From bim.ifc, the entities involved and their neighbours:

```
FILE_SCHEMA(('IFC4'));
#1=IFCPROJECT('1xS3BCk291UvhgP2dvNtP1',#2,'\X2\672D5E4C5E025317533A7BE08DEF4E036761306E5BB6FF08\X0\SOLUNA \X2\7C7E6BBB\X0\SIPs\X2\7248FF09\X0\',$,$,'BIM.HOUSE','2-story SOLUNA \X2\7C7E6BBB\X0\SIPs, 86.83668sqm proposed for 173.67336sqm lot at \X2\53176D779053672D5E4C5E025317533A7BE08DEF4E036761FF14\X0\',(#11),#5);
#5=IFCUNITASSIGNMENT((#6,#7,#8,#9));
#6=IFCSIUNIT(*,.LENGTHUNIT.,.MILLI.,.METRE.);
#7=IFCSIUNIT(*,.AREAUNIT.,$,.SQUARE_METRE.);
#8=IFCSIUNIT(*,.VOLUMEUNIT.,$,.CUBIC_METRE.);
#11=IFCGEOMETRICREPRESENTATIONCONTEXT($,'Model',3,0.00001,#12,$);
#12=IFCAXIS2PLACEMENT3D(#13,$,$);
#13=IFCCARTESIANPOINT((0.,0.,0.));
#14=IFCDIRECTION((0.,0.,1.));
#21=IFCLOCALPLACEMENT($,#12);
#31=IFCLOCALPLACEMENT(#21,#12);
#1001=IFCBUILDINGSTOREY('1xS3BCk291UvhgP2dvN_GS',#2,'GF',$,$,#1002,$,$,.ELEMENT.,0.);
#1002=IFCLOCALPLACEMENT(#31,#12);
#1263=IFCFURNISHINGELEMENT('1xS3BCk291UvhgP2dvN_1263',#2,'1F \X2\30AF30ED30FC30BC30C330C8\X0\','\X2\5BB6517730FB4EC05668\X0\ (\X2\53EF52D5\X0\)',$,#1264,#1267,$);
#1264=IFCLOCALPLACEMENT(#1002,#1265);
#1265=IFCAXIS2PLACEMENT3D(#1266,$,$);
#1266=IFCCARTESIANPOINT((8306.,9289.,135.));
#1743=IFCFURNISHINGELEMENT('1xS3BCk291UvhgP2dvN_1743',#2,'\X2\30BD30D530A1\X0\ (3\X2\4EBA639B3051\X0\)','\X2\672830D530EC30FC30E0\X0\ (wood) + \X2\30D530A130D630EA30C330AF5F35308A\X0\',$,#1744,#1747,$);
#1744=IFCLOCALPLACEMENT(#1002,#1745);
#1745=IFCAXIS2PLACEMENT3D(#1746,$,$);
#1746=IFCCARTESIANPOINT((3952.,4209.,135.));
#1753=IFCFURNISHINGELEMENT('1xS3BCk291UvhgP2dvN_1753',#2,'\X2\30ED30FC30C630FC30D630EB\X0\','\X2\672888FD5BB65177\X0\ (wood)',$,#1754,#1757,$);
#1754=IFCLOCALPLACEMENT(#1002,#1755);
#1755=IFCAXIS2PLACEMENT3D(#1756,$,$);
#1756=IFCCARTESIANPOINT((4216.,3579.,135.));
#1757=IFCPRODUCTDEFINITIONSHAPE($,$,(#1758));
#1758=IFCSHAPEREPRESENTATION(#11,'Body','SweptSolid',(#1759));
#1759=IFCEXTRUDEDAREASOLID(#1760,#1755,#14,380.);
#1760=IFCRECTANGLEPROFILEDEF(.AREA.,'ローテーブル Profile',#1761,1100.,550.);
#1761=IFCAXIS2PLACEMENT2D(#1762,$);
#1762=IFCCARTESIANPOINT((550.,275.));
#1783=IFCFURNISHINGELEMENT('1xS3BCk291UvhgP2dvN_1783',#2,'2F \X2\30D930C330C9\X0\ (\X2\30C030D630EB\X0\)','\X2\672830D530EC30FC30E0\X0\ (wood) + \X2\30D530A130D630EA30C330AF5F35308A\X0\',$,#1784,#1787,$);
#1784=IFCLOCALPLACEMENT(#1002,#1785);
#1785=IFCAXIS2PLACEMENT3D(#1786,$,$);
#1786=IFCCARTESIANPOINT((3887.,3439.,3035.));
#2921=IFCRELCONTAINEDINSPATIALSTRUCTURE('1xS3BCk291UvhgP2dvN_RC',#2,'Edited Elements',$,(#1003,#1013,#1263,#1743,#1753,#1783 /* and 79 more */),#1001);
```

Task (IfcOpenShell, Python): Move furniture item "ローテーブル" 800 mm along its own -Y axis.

```python
import ifcopenshell
import ifcopenshell.api.geometry
import ifcopenshell.util.placement
import ifcopenshell.util.unit

model = ifcopenshell.open("bim.ifc")
unit_scale = ifcopenshell.util.unit.calculate_unit_scale(model)

item = model.by_guid("1xS3BCk291UvhgP2dvN_1753")
matrix = ifcopenshell.util.placement.get_local_placement(item.ObjectPlacement)
matrix[:3, 3] -= matrix[:3, 1] * 0.8 / unit_scale
ifcopenshell.api.geometry.edit_object_placement(model, product=item, matrix=matrix, is_si=False)

print(ifcopenshell.util.placement.get_local_placement(item.ObjectPlacement).round(3) + 0.0)

model.write("bim-out.ifc")
```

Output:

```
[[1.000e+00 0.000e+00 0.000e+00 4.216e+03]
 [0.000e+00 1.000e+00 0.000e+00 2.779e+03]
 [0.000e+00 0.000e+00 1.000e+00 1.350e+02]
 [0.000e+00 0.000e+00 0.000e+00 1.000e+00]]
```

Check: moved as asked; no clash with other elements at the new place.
